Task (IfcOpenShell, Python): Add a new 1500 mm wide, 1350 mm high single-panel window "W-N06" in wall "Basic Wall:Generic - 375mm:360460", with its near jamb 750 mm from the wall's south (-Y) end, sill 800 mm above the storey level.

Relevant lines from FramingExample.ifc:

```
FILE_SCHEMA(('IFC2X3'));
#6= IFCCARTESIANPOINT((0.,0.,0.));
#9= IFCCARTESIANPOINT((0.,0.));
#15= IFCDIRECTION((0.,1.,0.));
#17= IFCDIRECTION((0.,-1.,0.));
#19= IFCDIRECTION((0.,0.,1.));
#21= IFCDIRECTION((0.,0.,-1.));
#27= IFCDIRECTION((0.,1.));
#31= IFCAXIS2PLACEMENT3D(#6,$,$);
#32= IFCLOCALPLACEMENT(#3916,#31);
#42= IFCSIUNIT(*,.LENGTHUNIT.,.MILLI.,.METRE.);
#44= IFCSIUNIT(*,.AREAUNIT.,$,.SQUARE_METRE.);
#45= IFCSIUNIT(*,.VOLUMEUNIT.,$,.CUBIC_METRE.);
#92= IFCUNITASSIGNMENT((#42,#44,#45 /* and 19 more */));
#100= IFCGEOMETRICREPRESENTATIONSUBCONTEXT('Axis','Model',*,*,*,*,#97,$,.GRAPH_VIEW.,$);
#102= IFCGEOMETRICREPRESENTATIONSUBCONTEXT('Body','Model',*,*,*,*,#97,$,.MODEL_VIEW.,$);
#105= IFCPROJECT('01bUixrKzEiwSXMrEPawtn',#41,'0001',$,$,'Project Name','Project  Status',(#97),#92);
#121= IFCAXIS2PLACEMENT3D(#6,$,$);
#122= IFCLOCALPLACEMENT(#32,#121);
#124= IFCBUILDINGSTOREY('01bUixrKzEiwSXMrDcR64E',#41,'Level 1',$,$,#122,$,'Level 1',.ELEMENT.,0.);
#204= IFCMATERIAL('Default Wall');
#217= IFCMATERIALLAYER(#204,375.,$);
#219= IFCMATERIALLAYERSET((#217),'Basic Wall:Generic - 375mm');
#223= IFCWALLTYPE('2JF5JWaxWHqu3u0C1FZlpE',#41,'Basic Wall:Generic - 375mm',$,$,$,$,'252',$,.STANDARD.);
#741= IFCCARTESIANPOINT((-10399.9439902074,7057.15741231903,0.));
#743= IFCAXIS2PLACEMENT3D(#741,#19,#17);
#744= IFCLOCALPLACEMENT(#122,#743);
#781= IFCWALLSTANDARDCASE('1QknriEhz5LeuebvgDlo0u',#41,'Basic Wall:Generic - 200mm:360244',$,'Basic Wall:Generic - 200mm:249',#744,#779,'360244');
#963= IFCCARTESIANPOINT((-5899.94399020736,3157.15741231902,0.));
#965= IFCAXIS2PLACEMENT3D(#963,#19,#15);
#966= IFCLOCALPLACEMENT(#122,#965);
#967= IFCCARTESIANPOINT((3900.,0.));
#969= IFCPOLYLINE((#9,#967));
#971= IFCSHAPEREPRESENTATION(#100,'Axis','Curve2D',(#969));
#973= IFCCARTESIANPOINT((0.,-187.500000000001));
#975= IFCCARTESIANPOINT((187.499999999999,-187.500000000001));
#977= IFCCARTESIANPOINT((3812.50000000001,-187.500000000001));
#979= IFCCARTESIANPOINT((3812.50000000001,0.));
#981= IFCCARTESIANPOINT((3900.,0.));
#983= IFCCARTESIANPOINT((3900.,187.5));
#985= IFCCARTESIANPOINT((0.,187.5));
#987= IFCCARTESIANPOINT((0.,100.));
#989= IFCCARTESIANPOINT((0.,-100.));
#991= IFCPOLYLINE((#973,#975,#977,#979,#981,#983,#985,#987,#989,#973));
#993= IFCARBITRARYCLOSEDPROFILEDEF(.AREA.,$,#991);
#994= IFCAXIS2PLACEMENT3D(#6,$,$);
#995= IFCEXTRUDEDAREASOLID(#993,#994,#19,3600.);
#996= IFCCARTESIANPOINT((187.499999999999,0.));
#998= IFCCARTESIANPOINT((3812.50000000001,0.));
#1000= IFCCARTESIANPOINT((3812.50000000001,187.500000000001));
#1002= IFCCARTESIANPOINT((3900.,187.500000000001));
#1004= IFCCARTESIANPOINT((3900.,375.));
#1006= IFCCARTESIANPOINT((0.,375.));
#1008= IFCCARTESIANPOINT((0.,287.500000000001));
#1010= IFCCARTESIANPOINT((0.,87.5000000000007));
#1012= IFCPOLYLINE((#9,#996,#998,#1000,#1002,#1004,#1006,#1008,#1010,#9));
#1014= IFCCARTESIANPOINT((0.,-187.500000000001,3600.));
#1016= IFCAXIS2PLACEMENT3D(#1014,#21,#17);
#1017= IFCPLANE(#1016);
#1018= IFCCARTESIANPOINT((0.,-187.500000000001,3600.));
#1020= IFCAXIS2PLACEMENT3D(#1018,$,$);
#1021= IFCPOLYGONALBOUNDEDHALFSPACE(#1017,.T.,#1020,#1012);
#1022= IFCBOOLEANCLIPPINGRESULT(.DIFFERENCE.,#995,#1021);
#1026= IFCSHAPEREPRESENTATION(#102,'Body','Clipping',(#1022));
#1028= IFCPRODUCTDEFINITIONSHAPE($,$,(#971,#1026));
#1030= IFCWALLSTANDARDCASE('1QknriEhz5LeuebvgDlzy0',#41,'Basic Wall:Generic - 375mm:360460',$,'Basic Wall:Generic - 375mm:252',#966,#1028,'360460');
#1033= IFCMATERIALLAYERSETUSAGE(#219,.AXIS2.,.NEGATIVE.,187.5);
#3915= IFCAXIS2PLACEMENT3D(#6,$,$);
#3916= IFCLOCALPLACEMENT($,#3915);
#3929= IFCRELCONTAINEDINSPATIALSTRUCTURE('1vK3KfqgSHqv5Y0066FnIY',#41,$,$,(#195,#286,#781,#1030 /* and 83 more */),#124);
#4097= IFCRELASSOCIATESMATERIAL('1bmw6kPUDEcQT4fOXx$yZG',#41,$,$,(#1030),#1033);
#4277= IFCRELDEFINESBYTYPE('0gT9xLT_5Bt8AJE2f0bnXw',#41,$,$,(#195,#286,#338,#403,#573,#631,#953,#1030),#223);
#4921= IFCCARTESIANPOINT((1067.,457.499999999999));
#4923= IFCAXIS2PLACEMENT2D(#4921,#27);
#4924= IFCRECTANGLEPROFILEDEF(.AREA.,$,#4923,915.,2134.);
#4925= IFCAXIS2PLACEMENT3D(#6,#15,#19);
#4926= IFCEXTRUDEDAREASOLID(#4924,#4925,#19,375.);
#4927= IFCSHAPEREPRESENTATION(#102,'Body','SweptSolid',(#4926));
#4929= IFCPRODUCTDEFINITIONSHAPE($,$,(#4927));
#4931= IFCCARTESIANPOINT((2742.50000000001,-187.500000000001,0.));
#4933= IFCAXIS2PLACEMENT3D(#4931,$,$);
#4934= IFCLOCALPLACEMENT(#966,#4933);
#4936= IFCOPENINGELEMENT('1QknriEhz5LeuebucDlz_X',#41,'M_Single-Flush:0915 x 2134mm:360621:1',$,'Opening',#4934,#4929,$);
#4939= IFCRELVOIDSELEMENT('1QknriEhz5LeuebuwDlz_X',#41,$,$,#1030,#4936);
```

```python
import numpy as np
import ifcopenshell
import ifcopenshell.api.feature
import ifcopenshell.api.geometry
import ifcopenshell.api.root
import ifcopenshell.api.spatial
import ifcopenshell.api.type
import ifcopenshell.geom
import ifcopenshell.util.element
import ifcopenshell.util.placement
import ifcopenshell.util.representation
import ifcopenshell.util.shape
import ifcopenshell.util.unit

model = ifcopenshell.open("FramingExample.ifc")
unit_scale = ifcopenshell.util.unit.calculate_unit_scale(model)
settings = ifcopenshell.geom.settings()


def volume(element):
    """Net volume in cubic metres, openings subtracted."""
    shape = ifcopenshell.geom.create_shape(settings, element)
    return ifcopenshell.util.shape.get_volume(shape.geometry)


wall = model.by_guid("1QknriEhz5LeuebvgDlzy0")
storey = ifcopenshell.util.element.get_container(wall, ifc_class="IfcBuildingStorey")
context = ifcopenshell.util.representation.get_context(model, "Model", "Body", "MODEL_VIEW")
before = volume(wall)

width, height, from_end, sill = 1.5, 1.35, 0.75, 0.8  # metres

# The wall runs along its own X axis, and the end named is its -X end.
wall_shape = ifcopenshell.geom.create_shape(settings, wall)
x, y, z = ifcopenshell.util.shape.get_vertices(wall_shape.geometry).T
start = x.min() + from_end
face, thickness = float(y.min()), float(y.max() - y.min())
wall_matrix = ifcopenshell.util.placement.get_local_placement(wall.ObjectPlacement)
level = ifcopenshell.util.placement.get_local_placement(storey.ObjectPlacement)[2, 3]


def in_wall(x, y):
    """Placement at x, y metres in the wall's axes, at sill height."""
    matrix = wall_matrix.copy()
    matrix[:, 3] = wall_matrix @ np.array([x / unit_scale, y / unit_scale, 0.0, 1.0])
    matrix[2, 3] = level + sill / unit_scale
    return matrix


# Opening: a box that overshoots both wall faces by 50 mm.
opening = ifcopenshell.api.root.create_entity(model, ifc_class="IfcOpeningElement")
box = ifcopenshell.api.geometry.add_wall_representation(
    model, context=context, length=width, height=height, thickness=thickness + 0.1
)
ifcopenshell.api.geometry.assign_representation(model, product=opening, representation=box)
ifcopenshell.api.geometry.edit_object_placement(model, product=opening, matrix=in_wall(start, face - 0.05), is_si=False)
ifcopenshell.api.feature.add_feature(model, feature=opening, element=wall)

window = ifcopenshell.api.root.create_entity(model, ifc_class="IfcWindow", name="W-N06")
window.OverallWidth, window.OverallHeight = width / unit_scale, height / unit_scale
body = ifcopenshell.api.geometry.add_window_representation(
    model,
    context=context,
    overall_width=window.OverallWidth,
    overall_height=window.OverallHeight,
    partition_type="SINGLE_PANEL",
)
ifcopenshell.api.geometry.assign_representation(model, product=window, representation=body)
ifcopenshell.api.spatial.assign_container(model, products=[window], relating_structure=storey)
fills = ifcopenshell.api.feature.add_filling(model, opening=opening, element=window)
fills.OwnerHistory = window.OwnerHistory  # required in IFC2X3

# IFC2X3 keeps the operation on the window style.
style = ifcopenshell.api.root.create_entity(model, ifc_class="IfcWindowStyle", name="W-N06")
style.OperationType, style.ConstructionType = "SINGLE_PANEL", "NOTDEFINED"
style.ParameterTakesPrecedence = style.Sizeable = False
ifcopenshell.api.type.assign_type(model, related_objects=[window], relating_type=style)

# Centre the window in the wall's thickness.
ifcopenshell.api.geometry.edit_object_placement(model, product=window, matrix=in_wall(start, face), is_si=False)
window_shape = ifcopenshell.geom.create_shape(settings, window)
depth = ifcopenshell.util.shape.get_vertices(window_shape.geometry)[:, 1]
offset = face + thickness / 2 - (depth.min() + depth.max()) / 2
ifcopenshell.api.geometry.edit_object_placement(model, product=window, matrix=in_wall(start, offset), is_si=False)

after = volume(wall)

print(f"wall volume {before:.3f} -> {after:.3f} m3")

model.write("FramingExample_edited.ifc")
```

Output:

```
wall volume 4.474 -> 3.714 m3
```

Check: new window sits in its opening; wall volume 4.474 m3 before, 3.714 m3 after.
